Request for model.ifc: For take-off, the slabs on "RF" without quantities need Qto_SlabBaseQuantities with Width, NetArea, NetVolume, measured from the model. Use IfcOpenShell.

First a look at what the model holds.

```python
import ifcopenshell
import ifcopenshell.util.element
import ifcopenshell.util.unit

model = ifcopenshell.open("model.ifc")
print(model.schema)
for unit_type in ("LENGTHUNIT", "AREAUNIT", "VOLUMEUNIT"):
    print(unit_type, ifcopenshell.util.unit.calculate_unit_scale(model, unit_type))
storey = next(s for s in model.by_type("IfcBuildingStorey") if s.Name == "RF")
slabs = [e for e in ifcopenshell.util.element.get_decomposition(storey) if e.is_a("IfcSlab")]
for e in sorted(slabs, key=lambda e: e.id()):
    print(e.id(), e.is_a(), e.Name, list(ifcopenshell.util.element.get_psets(e, qtos_only=True)), sep=" | ")
```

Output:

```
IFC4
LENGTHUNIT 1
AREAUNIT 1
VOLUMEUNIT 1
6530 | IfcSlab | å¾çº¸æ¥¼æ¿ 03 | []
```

```python
import ifcopenshell
import ifcopenshell.api.pset
import ifcopenshell.geom
import ifcopenshell.util.element
import ifcopenshell.util.shape
import ifcopenshell.util.unit

model = ifcopenshell.open("model.ifc")
unit_scale = ifcopenshell.util.unit.calculate_unit_scale(model)
area_scale = ifcopenshell.util.unit.calculate_unit_scale(model, "AREAUNIT")
volume_scale = ifcopenshell.util.unit.calculate_unit_scale(model, "VOLUMEUNIT")
settings = ifcopenshell.geom.settings()

storey = next(s for s in model.by_type("IfcBuildingStorey") if s.Name == "RF")
slabs = [e for e in ifcopenshell.util.element.get_decomposition(storey) if e.is_a("IfcSlab")]

for e in sorted(slabs, key=lambda e: e.id()):
    if ifcopenshell.util.element.get_psets(e, qtos_only=True, should_inherit=False):
        continue
    # Geometry comes back in metres, in the element's own axes.
    shape = ifcopenshell.geom.create_shape(settings, e)
    values = {
        "Width": ifcopenshell.util.shape.get_z(shape.geometry) / unit_scale,
        "NetArea": ifcopenshell.util.shape.get_footprint_area(shape.geometry) / area_scale,
        "NetVolume": ifcopenshell.util.shape.get_volume(shape.geometry) / volume_scale,
    }
    qto = ifcopenshell.api.pset.add_qto(model, product=e, name="Qto_SlabBaseQuantities")
    ifcopenshell.api.pset.edit_qto(model, qto=qto, properties=values)
    print(e.id(), {k: round(v, 3) for k, v in values.items()})

model.write("model_rev.ifc")
```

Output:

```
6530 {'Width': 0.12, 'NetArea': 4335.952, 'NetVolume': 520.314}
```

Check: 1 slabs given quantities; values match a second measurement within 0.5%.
